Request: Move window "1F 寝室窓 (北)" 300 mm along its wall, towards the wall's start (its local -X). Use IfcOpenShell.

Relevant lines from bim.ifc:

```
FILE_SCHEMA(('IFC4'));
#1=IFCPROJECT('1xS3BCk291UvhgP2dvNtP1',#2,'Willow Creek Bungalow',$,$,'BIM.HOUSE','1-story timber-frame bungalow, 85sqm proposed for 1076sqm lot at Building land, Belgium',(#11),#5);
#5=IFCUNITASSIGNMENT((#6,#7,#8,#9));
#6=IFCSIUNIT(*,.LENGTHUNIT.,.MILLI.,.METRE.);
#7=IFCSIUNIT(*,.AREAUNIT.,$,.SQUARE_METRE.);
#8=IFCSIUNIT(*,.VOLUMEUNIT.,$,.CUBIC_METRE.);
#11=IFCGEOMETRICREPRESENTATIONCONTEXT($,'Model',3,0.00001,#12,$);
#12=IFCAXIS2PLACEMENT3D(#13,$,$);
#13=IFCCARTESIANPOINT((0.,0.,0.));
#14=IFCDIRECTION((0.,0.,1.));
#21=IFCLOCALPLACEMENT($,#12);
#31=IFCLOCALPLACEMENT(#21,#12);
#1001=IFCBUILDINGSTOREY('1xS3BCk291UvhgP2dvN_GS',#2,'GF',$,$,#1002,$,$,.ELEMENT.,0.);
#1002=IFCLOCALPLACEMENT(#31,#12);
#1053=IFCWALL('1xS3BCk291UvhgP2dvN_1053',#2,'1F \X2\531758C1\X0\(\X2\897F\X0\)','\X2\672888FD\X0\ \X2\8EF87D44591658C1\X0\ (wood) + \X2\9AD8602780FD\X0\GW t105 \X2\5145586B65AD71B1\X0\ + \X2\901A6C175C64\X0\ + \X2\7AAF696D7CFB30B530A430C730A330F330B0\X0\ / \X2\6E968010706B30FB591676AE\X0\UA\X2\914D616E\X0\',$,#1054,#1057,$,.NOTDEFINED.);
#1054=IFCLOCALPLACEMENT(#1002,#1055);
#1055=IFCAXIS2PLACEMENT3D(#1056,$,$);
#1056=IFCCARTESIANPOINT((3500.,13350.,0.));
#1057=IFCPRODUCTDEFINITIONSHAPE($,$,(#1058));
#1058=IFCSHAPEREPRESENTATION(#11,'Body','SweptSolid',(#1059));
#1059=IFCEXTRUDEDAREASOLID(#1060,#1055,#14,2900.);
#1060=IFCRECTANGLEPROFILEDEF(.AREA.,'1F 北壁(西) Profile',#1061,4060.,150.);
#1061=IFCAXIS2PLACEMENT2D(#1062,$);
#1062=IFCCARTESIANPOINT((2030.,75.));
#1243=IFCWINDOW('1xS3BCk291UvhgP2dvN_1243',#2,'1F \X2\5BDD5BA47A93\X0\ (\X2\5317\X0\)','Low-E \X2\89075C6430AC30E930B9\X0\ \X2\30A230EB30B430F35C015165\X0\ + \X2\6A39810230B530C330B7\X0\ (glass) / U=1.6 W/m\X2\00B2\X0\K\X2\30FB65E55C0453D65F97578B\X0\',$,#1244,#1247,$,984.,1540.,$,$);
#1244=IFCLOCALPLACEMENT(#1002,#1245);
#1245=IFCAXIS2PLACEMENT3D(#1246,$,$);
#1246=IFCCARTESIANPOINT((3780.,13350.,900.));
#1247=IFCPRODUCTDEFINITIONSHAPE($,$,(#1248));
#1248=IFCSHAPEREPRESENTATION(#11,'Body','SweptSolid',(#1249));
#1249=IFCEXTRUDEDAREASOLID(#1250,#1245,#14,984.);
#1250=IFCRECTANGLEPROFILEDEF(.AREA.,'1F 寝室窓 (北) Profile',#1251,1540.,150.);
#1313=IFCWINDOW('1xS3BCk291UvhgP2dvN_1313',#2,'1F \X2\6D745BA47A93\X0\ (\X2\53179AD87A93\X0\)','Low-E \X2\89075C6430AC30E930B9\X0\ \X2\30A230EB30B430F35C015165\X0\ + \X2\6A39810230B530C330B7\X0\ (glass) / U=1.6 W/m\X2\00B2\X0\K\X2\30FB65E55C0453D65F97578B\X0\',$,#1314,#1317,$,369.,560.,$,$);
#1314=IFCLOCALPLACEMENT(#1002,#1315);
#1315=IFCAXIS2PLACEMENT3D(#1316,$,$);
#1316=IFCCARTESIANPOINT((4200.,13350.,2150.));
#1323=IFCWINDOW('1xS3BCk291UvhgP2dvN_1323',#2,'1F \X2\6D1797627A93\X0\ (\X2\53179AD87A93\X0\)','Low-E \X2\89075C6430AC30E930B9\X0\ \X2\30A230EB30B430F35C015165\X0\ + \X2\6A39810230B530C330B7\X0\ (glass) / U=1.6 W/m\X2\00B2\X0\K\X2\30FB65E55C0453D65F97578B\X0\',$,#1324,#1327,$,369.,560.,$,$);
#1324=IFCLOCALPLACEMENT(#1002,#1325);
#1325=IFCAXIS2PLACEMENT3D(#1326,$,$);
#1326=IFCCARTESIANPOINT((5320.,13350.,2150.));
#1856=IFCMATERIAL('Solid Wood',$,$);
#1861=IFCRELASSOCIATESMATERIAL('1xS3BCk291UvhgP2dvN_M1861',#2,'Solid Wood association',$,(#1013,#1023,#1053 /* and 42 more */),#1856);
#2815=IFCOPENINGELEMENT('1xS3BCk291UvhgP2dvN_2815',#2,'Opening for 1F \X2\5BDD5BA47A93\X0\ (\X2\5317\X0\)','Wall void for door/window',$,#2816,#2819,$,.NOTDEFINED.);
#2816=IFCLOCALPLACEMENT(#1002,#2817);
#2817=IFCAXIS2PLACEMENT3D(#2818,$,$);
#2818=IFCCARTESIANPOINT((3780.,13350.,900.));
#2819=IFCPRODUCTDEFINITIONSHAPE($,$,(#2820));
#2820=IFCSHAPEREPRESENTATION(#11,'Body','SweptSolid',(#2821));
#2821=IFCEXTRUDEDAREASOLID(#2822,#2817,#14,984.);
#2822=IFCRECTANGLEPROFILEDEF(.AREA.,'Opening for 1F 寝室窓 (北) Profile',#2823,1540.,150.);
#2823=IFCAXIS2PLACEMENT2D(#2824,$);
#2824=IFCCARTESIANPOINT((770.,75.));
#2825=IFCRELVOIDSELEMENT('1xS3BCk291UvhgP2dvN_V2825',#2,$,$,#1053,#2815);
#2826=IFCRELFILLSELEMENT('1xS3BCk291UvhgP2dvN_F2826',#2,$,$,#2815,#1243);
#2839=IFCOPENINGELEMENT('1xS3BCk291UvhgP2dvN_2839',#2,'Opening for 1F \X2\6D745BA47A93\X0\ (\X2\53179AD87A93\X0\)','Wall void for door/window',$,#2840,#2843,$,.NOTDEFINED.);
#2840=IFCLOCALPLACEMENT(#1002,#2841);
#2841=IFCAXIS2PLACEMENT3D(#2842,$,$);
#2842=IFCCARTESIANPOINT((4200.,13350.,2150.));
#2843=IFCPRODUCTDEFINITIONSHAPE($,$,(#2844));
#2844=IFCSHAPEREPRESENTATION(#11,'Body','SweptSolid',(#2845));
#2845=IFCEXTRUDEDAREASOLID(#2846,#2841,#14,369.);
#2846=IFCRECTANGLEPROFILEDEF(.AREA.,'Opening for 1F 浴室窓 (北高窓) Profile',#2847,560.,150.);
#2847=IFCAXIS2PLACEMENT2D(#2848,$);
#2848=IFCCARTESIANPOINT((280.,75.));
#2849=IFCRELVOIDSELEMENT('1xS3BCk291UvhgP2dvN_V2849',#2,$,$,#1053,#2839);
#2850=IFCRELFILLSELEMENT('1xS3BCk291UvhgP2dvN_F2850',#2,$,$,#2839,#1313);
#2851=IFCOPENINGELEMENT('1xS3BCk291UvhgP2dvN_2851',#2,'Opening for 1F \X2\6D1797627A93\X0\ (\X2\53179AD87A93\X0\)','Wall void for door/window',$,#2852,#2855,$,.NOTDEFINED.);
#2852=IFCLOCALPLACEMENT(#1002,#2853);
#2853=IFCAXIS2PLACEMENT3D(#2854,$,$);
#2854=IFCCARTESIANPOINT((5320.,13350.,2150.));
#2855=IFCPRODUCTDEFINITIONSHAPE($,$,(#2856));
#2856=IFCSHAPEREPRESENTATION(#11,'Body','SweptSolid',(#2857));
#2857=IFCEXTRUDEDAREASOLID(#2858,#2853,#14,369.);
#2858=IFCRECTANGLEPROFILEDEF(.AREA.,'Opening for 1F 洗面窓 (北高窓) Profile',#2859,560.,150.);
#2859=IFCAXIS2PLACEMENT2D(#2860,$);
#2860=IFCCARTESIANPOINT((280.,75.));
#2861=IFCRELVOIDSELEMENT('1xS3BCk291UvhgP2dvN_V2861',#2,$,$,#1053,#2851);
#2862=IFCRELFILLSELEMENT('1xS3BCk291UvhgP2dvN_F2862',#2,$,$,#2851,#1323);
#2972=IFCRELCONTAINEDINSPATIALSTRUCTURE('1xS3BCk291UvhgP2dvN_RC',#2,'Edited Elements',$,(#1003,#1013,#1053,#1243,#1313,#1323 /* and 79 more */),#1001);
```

```python
import ifcopenshell
import ifcopenshell.api.geometry
import ifcopenshell.util.placement
import ifcopenshell.util.unit

model = ifcopenshell.open("bim.ifc")
unit_scale = ifcopenshell.util.unit.calculate_unit_scale(model)

window = model.by_id(1243)
opening = window.FillsVoids[0].RelatingOpeningElement
wall = opening.VoidsElements[0].RelatingBuildingElement

wall_matrix = ifcopenshell.util.placement.get_local_placement(wall.ObjectPlacement)
shift = wall_matrix[:3, 0] * -0.3 / unit_scale
before = ifcopenshell.util.placement.get_local_placement(window.ObjectPlacement)[:3, 3].copy()

# The window is not placed relative to its opening, so move both.
for product in (opening, window):
    matrix = ifcopenshell.util.placement.get_local_placement(product.ObjectPlacement)
    matrix[:3, 3] += shift
    ifcopenshell.api.geometry.edit_object_placement(model, product=product, matrix=matrix, is_si=False)

after = ifcopenshell.util.placement.get_local_placement(window.ObjectPlacement)[:3, 3]
print("window moved by", (after - before).round(3) + 0.0)

model.write("bim_edited.ifc")
```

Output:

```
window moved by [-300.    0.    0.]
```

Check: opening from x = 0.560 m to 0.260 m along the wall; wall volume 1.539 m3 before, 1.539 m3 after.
